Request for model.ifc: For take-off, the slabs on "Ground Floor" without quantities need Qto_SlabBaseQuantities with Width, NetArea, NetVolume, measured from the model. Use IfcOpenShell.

First a look at what the model holds.

```python
import ifcopenshell
import ifcopenshell.util.element
import ifcopenshell.util.unit

model = ifcopenshell.open("model.ifc")
print(model.schema)
for unit_type in ("LENGTHUNIT", "AREAUNIT", "VOLUMEUNIT"):
    print(unit_type, ifcopenshell.util.unit.calculate_unit_scale(model, unit_type))
storey = next(s for s in model.by_type("IfcBuildingStorey") if s.Name == "Ground Floor")
slabs = [e for e in ifcopenshell.util.element.get_decomposition(storey) if e.is_a("IfcSlab")]
for e in sorted(slabs, key=lambda e: e.id()):
    print(e.id(), e.is_a(), e.Name, list(ifcopenshell.util.element.get_psets(e, qtos_only=True)), sep=" | ")
```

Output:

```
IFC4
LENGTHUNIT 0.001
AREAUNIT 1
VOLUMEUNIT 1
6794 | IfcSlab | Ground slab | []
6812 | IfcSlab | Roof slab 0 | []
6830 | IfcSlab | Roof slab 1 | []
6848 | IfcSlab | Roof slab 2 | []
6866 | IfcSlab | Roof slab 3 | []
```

```python
import ifcopenshell
import ifcopenshell.api.pset
import ifcopenshell.geom
import ifcopenshell.util.element
import ifcopenshell.util.shape
import ifcopenshell.util.unit

model = ifcopenshell.open("model.ifc")
unit_scale = ifcopenshell.util.unit.calculate_unit_scale(model)
area_scale = ifcopenshell.util.unit.calculate_unit_scale(model, "AREAUNIT")
volume_scale = ifcopenshell.util.unit.calculate_unit_scale(model, "VOLUMEUNIT")
settings = ifcopenshell.geom.settings()

storey = next(s for s in model.by_type("IfcBuildingStorey") if s.Name == "Ground Floor")
slabs = [e for e in ifcopenshell.util.element.get_decomposition(storey) if e.is_a("IfcSlab")]

for e in sorted(slabs, key=lambda e: e.id()):
    if ifcopenshell.util.element.get_psets(e, qtos_only=True, should_inherit=False):
        continue
    # Geometry comes back in metres, in the element's own axes.
    shape = ifcopenshell.geom.create_shape(settings, e)
    values = {
        "Width": ifcopenshell.util.shape.get_z(shape.geometry) / unit_scale,
        "NetArea": ifcopenshell.util.shape.get_footprint_area(shape.geometry) / area_scale,
        "NetVolume": ifcopenshell.util.shape.get_volume(shape.geometry) / volume_scale,
    }
    qto = ifcopenshell.api.pset.add_qto(model, product=e, name="Qto_SlabBaseQuantities")
    ifcopenshell.api.pset.edit_qto(model, qto=qto, properties=values)
    print(e.id(), {k: round(v, 3) for k, v in values.items()})

model.write("model-out.ifc")
```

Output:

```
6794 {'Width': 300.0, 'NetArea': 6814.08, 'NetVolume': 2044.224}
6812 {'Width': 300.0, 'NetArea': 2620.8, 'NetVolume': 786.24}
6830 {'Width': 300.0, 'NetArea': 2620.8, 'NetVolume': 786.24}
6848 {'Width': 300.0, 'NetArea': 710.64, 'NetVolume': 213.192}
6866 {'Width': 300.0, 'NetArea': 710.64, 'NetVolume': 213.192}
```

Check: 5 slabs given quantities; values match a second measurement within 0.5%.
